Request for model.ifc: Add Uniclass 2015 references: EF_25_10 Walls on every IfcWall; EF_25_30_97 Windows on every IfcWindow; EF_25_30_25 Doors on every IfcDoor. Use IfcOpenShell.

First a look at what the model holds.

```python
import ifcopenshell

model = ifcopenshell.open("model.ifc")
print(model.schema)
print("classifications:", [c.Name for c in model.by_type("IfcClassification")])
for ifc_class in ("IfcDoor", "IfcRoof", "IfcStair", "IfcWall", "IfcWindow"):
    print(ifc_class, len(model.by_type(ifc_class)))
```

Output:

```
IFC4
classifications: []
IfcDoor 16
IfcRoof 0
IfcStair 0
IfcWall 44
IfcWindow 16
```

```python
import ifcopenshell
import ifcopenshell.api.classification

model = ifcopenshell.open("model.ifc")

system = ifcopenshell.api.classification.add_classification(model, classification="Uniclass 2015")

codes = {
    "IfcWall": ("EF_25_10", "Walls"),
    "IfcWindow": ("EF_25_30_97", "Windows"),
    "IfcDoor": ("EF_25_30_25", "Doors"),
}
for ifc_class, (code, name) in codes.items():
    products = model.by_type(ifc_class)
    ifcopenshell.api.classification.add_reference(
        model, products=products, classification=system, identification=code, name=name
    )
    print(code, len(products))

model.write("model-out.ifc")
```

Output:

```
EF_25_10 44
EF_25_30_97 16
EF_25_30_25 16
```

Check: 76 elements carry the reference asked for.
